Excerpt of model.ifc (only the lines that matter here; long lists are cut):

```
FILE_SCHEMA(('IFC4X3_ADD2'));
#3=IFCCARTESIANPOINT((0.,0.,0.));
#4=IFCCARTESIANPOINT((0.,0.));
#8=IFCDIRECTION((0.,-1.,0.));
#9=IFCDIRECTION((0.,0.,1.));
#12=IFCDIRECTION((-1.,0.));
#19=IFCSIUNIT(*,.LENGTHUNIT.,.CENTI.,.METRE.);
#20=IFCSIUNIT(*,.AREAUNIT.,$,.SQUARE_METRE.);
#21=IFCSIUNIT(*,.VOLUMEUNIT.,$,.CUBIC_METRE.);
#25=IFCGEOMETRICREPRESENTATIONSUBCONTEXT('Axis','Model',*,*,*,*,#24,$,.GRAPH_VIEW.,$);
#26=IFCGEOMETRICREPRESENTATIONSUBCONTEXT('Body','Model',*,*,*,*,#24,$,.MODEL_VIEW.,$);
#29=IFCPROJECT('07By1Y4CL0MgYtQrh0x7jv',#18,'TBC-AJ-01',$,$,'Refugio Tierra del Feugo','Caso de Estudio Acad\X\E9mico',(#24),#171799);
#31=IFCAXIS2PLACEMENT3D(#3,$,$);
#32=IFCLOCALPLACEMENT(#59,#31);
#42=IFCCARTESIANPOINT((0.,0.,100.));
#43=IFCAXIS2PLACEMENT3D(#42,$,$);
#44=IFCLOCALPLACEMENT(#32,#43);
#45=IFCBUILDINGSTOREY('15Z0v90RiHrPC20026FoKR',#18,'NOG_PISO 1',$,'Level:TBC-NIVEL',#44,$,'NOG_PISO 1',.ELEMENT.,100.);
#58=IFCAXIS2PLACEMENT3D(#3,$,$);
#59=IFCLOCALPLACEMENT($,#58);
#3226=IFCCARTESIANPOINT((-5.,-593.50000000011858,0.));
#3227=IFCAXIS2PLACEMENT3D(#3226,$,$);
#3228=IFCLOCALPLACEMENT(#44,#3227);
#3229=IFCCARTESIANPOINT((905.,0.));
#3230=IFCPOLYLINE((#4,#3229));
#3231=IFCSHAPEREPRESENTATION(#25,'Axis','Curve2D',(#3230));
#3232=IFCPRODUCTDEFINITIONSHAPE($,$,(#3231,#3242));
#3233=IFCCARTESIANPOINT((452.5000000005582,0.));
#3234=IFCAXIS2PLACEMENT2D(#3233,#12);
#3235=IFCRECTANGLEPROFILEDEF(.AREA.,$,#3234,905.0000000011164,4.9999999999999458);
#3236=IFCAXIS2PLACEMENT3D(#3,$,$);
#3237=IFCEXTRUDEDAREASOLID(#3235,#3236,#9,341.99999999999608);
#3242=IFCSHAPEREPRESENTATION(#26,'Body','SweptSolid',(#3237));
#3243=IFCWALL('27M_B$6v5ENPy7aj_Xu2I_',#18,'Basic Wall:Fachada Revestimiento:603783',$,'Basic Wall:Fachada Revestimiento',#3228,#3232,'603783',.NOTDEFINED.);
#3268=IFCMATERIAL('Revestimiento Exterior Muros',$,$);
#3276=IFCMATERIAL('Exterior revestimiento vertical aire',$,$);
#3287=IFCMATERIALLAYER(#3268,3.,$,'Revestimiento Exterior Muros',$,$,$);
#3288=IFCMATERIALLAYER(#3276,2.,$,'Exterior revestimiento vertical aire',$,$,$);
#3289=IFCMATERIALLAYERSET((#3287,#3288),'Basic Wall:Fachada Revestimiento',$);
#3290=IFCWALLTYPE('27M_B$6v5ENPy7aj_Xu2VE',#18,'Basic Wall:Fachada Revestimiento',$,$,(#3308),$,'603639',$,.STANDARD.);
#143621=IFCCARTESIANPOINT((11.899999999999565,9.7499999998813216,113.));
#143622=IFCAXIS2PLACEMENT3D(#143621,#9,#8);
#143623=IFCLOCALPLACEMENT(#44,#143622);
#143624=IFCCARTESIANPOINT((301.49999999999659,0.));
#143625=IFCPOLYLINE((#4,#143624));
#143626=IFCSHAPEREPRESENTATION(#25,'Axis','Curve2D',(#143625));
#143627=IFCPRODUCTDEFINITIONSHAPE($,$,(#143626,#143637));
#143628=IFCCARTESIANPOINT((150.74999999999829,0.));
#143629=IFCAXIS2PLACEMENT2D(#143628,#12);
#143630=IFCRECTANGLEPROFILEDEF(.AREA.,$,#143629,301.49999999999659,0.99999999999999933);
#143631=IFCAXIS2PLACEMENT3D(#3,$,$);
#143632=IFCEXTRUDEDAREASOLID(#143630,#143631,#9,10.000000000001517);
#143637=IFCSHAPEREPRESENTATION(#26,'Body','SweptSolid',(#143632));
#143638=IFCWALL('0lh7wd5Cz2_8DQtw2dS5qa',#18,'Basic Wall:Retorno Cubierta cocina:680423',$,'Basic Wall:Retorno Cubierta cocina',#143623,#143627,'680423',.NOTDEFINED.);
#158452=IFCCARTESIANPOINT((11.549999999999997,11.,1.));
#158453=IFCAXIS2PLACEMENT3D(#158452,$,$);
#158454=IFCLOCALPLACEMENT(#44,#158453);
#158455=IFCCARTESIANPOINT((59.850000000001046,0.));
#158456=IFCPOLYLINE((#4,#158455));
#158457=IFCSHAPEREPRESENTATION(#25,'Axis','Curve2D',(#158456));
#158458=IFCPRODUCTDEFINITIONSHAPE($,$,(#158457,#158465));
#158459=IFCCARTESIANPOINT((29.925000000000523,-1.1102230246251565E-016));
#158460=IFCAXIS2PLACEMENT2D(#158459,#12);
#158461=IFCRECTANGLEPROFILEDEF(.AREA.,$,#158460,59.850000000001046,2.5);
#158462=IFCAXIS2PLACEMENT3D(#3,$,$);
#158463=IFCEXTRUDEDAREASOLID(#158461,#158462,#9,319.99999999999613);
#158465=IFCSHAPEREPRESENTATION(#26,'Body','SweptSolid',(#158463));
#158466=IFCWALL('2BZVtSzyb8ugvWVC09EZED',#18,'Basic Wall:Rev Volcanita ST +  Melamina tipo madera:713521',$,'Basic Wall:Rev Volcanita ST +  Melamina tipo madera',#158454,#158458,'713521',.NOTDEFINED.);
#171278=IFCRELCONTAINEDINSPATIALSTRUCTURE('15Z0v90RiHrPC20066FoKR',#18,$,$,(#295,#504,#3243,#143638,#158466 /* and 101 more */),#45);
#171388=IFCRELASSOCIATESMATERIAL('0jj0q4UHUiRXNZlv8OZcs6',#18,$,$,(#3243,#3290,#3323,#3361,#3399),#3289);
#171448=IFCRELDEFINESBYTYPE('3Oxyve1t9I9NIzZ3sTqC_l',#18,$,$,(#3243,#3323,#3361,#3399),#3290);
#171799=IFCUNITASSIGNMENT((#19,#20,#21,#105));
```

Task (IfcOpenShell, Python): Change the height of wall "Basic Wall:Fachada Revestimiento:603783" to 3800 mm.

```python
import ifcopenshell
import ifcopenshell.geom
import ifcopenshell.util.representation
import ifcopenshell.util.shape
import ifcopenshell.util.unit

model = ifcopenshell.open("model.ifc")
unit_scale = ifcopenshell.util.unit.calculate_unit_scale(model)
settings = ifcopenshell.geom.settings()


def volume(element):
    """Net volume in cubic metres, openings subtracted."""
    shape = ifcopenshell.geom.create_shape(settings, element)
    return ifcopenshell.util.shape.get_volume(shape.geometry)


wall = model.by_id(3243)
before = volume(wall)

body = ifcopenshell.util.representation.get_representation(wall, "Model", "Body")
solid = body.Items[0]
old_height = solid.Depth
solid.Depth = 3.8 / unit_scale
after = volume(wall)

print(f"height {old_height:g} -> {solid.Depth:g}, volume {before:.3f} -> {after:.3f} m3")

model.write("model-out.ifc")
```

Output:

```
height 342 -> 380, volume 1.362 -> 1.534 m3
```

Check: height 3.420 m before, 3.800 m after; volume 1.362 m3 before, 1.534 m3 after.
